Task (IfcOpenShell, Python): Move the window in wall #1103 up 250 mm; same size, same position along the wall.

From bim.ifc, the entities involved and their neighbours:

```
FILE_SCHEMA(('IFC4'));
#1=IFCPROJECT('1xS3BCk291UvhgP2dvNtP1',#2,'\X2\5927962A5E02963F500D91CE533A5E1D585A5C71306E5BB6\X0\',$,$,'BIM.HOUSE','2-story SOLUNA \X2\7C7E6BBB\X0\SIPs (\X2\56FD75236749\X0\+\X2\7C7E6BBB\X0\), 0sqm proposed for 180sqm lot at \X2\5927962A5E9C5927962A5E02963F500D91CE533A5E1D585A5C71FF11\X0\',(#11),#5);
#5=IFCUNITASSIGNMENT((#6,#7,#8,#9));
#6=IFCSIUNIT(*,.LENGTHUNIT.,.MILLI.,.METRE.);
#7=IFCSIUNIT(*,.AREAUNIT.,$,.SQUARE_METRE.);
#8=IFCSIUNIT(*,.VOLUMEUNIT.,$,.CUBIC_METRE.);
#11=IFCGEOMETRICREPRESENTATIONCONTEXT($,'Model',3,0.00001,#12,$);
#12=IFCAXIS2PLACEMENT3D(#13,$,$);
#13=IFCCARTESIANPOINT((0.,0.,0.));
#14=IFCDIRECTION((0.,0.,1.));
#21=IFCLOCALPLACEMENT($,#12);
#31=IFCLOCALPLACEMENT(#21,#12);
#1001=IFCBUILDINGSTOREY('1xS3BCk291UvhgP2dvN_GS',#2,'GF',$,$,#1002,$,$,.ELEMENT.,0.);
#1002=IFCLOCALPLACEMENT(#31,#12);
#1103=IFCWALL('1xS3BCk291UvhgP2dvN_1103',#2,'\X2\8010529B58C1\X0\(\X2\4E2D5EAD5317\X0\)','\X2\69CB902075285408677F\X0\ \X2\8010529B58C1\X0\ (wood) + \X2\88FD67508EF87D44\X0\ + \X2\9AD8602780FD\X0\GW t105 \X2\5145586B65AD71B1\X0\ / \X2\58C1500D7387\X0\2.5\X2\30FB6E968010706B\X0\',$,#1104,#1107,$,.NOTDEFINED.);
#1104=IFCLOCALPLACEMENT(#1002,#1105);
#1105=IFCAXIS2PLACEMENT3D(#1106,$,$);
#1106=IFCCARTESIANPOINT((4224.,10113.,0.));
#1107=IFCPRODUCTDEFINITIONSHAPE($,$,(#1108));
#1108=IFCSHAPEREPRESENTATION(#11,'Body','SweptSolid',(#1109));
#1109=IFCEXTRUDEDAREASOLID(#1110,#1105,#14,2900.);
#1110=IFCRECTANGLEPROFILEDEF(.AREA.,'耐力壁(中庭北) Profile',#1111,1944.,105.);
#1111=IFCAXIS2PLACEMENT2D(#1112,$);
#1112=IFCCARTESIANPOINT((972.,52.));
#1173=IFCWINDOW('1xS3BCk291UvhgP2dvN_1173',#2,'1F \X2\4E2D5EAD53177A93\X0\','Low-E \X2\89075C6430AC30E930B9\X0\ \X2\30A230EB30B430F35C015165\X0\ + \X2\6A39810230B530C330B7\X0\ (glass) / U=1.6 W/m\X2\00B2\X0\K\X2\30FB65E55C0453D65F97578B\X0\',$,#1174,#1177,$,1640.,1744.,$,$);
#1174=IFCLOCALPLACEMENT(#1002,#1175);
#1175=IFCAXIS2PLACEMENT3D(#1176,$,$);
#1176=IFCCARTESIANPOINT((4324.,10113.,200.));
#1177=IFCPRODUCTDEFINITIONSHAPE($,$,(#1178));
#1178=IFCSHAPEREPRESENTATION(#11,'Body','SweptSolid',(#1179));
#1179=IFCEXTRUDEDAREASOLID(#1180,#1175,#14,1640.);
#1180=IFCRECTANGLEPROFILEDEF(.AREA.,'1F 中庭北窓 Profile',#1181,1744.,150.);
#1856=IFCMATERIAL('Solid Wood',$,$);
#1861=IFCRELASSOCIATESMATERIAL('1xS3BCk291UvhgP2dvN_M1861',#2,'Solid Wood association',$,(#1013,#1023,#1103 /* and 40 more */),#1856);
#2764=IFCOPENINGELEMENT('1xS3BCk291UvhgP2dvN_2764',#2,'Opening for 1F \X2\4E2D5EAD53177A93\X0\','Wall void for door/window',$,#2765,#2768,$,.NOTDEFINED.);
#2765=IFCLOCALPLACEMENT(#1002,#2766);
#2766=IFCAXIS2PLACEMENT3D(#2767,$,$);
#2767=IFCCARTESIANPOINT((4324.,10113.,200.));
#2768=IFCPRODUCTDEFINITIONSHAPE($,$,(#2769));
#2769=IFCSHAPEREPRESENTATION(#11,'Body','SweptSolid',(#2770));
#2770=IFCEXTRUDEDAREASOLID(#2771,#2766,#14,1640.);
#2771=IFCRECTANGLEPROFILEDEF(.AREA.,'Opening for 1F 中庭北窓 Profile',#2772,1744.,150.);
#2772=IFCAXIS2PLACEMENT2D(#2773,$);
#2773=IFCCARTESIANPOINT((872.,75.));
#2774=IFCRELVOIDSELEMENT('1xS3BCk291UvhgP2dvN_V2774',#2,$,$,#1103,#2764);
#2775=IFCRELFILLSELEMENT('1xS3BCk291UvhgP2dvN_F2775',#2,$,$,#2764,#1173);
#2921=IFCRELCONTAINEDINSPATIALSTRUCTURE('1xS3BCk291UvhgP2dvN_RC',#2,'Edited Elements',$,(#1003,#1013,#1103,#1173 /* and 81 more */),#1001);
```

```python
import numpy as np
import ifcopenshell
import ifcopenshell.api.geometry
import ifcopenshell.util.placement
import ifcopenshell.util.unit

model = ifcopenshell.open("bim.ifc")
unit_scale = ifcopenshell.util.unit.calculate_unit_scale(model)

window = model.by_id(1173)
opening = window.FillsVoids[0].RelatingOpeningElement
dz = 250.0

shift = np.array([0.0, 0.0, dz])
# The window is not placed relative to its opening, so move both.
for product in (opening, window):
    matrix = ifcopenshell.util.placement.get_local_placement(product.ObjectPlacement)
    matrix[:3, 3] += shift
    ifcopenshell.api.geometry.edit_object_placement(model, product=product, matrix=matrix, is_si=False)

print(f"moved by {dz * unit_scale:+.3f} m")

model.write("bim-out.ifc")
```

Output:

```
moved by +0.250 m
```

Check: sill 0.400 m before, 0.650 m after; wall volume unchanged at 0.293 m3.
